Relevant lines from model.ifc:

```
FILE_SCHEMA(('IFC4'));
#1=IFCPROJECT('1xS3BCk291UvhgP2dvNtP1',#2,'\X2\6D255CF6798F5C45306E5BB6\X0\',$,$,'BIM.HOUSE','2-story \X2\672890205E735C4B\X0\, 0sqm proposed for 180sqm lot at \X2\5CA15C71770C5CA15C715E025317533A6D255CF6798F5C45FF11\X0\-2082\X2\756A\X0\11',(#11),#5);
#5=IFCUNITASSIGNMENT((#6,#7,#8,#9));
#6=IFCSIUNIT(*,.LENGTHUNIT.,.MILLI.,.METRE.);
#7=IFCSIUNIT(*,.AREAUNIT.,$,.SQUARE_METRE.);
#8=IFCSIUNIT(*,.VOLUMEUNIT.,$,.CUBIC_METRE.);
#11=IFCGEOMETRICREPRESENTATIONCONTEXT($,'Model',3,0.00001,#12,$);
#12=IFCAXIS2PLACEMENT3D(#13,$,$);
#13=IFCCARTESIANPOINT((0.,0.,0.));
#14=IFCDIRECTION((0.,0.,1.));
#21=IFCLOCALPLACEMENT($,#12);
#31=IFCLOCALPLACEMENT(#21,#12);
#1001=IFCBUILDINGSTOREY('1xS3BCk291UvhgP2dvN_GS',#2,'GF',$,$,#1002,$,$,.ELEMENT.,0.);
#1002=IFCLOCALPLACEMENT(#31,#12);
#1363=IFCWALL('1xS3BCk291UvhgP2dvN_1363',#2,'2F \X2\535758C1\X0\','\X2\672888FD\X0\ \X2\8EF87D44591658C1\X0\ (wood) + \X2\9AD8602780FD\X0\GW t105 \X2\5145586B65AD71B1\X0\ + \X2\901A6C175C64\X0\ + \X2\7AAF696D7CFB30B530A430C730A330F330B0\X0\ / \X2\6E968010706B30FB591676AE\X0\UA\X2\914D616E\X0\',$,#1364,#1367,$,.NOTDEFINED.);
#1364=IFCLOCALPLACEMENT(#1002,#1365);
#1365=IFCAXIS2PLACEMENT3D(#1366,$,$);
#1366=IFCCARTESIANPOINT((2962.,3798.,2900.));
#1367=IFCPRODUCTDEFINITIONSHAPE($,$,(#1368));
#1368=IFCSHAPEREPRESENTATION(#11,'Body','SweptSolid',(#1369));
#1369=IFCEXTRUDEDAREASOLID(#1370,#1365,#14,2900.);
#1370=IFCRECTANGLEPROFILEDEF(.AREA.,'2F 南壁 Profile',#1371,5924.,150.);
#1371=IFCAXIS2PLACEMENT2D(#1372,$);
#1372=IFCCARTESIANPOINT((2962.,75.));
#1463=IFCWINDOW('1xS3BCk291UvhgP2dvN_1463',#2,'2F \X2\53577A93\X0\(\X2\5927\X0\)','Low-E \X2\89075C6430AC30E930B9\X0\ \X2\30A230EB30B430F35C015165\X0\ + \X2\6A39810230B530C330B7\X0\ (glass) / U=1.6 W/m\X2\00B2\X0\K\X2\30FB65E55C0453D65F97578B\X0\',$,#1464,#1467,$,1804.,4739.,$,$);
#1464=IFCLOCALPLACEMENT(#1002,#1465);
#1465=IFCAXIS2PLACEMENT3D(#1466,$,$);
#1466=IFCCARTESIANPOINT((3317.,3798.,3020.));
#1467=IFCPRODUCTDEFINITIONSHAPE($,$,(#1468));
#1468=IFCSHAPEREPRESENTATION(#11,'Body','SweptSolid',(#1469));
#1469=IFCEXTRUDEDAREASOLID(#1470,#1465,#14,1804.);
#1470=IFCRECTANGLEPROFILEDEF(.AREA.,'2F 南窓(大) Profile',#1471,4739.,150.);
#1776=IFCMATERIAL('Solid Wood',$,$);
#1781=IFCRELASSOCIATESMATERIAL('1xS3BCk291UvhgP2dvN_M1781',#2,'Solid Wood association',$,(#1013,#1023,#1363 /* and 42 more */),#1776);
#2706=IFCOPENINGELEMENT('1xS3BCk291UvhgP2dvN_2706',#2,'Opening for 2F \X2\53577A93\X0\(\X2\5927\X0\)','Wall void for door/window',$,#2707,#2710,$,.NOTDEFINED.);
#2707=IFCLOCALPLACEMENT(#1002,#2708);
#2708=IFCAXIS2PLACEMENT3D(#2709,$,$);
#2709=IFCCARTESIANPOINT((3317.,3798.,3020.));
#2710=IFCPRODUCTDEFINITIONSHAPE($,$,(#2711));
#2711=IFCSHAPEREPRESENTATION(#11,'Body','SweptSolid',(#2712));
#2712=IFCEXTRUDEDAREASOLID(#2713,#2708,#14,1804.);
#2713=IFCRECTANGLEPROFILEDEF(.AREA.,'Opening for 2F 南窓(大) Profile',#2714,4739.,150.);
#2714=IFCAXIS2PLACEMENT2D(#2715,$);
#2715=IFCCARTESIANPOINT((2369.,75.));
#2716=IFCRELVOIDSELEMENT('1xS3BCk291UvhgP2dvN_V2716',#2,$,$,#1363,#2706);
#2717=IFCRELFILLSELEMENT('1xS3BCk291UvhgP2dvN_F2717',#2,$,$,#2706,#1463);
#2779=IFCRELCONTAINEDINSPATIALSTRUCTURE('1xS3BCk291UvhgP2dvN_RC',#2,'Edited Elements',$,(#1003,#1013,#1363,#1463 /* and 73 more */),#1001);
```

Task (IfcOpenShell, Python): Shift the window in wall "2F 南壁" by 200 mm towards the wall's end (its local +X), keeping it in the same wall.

```python
import ifcopenshell
import ifcopenshell.api.geometry
import ifcopenshell.util.placement

model = ifcopenshell.open("model.ifc")

window = model.by_id(1463)
opening = window.FillsVoids[0].RelatingOpeningElement
wall = opening.VoidsElements[0].RelatingBuildingElement

wall_matrix = ifcopenshell.util.placement.get_local_placement(wall.ObjectPlacement)
shift = wall_matrix[:3, 0] * 200.0
before = ifcopenshell.util.placement.get_local_placement(window.ObjectPlacement)[:3, 3].copy()

# The window is not placed relative to its opening, so move both.
for product in (opening, window):
    matrix = ifcopenshell.util.placement.get_local_placement(product.ObjectPlacement)
    matrix[:3, 3] += shift
    ifcopenshell.api.geometry.edit_object_placement(model, product=product, matrix=matrix, is_si=False)

after = ifcopenshell.util.placement.get_local_placement(window.ObjectPlacement)[:3, 3]
print("window moved by", (after - before).round(3) + 0.0)

model.write("model-out.ifc")
```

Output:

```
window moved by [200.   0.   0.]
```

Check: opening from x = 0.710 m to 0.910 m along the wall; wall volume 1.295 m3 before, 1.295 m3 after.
